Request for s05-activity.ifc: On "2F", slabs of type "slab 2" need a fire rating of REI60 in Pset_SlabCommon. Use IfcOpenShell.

First a look at what the model holds.

```python
import ifcopenshell
import ifcopenshell.util.element

model = ifcopenshell.open("s05-activity.ifc")
print(model.schema)
storey = next(s for s in model.by_type("IfcBuildingStorey") if s.Name == "2F")
slabs = [e for e in ifcopenshell.util.element.get_decomposition(storey) if e.is_a("IfcSlab")]
seen = {}
for e in slabs:
    element_type = ifcopenshell.util.element.get_type(e)
    key = (element_type.Name if element_type != e and element_type else None, ifcopenshell.util.element.get_pset(e, "Pset_SlabCommon", "FireRating"))
    seen[key] = seen.get(key, 0) + 1
for (name, value), count in sorted(seen.items(), key=str):
    print(count, "x", name, "|", value)
```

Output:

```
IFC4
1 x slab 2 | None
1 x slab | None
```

```python
import ifcopenshell
import ifcopenshell.api.pset
import ifcopenshell.util.element

model = ifcopenshell.open("s05-activity.ifc")

storey = next(s for s in model.by_type("IfcBuildingStorey") if s.Name == "2F")
slabs = [e for e in ifcopenshell.util.element.get_decomposition(storey) if e.is_a("IfcSlab")]

count = 0
for e in slabs:
    element_type = ifcopenshell.util.element.get_type(e)
    if element_type in (None, e) or element_type.Name != "slab 2":
        continue
    # add_pset returns the element's existing set when there is one.
    pset = ifcopenshell.api.pset.add_pset(model, product=e, name="Pset_SlabCommon")
    ifcopenshell.api.pset.edit_pset(model, pset=pset, properties={"FireRating": "REI60"})
    count += 1

print(count, "slabs updated")

model.write("s05-activity_v2.ifc")
```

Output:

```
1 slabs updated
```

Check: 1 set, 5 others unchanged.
